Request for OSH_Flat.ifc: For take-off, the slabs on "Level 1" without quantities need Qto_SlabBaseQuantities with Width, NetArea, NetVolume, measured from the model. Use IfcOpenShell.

First a look at what the model holds.

```python
import ifcopenshell
import ifcopenshell.util.element
import ifcopenshell.util.unit

model = ifcopenshell.open("OSH_Flat.ifc")
print(model.schema)
for unit_type in ("LENGTHUNIT", "AREAUNIT", "VOLUMEUNIT"):
    print(unit_type, ifcopenshell.util.unit.calculate_unit_scale(model, unit_type))
storey = next(s for s in model.by_type("IfcBuildingStorey") if s.Name == "Level 1")
slabs = [e for e in ifcopenshell.util.element.get_decomposition(storey) if e.is_a("IfcSlab")]
for e in sorted(slabs, key=lambda e: e.id()):
    print(e.id(), e.is_a(), e.Name, list(ifcopenshell.util.element.get_psets(e, qtos_only=True)), sep=" | ")
```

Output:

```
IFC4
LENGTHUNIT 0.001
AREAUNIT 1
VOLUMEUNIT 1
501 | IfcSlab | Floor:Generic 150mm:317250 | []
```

```python
import ifcopenshell
import ifcopenshell.api.pset
import ifcopenshell.geom
import ifcopenshell.util.element
import ifcopenshell.util.shape
import ifcopenshell.util.unit

model = ifcopenshell.open("OSH_Flat.ifc")
unit_scale = ifcopenshell.util.unit.calculate_unit_scale(model)
area_scale = ifcopenshell.util.unit.calculate_unit_scale(model, "AREAUNIT")
volume_scale = ifcopenshell.util.unit.calculate_unit_scale(model, "VOLUMEUNIT")
settings = ifcopenshell.geom.settings()

storey = next(s for s in model.by_type("IfcBuildingStorey") if s.Name == "Level 1")
slabs = [e for e in ifcopenshell.util.element.get_decomposition(storey) if e.is_a("IfcSlab")]

for e in sorted(slabs, key=lambda e: e.id()):
    if ifcopenshell.util.element.get_psets(e, qtos_only=True, should_inherit=False):
        continue
    # Geometry comes back in metres, in the element's own axes.
    shape = ifcopenshell.geom.create_shape(settings, e)
    values = {
        "Width": ifcopenshell.util.shape.get_z(shape.geometry) / unit_scale,
        "NetArea": ifcopenshell.util.shape.get_footprint_area(shape.geometry) / area_scale,
        "NetVolume": ifcopenshell.util.shape.get_volume(shape.geometry) / volume_scale,
    }
    qto = ifcopenshell.api.pset.add_qto(model, product=e, name="Qto_SlabBaseQuantities")
    ifcopenshell.api.pset.edit_qto(model, qto=qto, properties=values)
    print(e.id(), {k: round(v, 3) for k, v in values.items()})

model.write("OSH_Flat-out.ifc")
```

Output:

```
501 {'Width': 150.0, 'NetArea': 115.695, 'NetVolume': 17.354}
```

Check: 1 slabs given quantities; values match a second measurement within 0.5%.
